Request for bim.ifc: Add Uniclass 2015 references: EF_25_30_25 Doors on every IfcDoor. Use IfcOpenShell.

First a look at what the model holds.

```python
import ifcopenshell

model = ifcopenshell.open("bim.ifc")
print(model.schema)
print("classifications:", [c.Name for c in model.by_type("IfcClassification")])
for ifc_class in ("IfcDoor", "IfcRoof", "IfcStair", "IfcWall", "IfcWindow"):
    print(ifc_class, len(model.by_type(ifc_class)))
```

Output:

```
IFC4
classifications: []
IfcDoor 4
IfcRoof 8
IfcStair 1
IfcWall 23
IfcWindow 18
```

```python
import ifcopenshell
import ifcopenshell.api.classification

model = ifcopenshell.open("bim.ifc")

system = ifcopenshell.api.classification.add_classification(model, classification="Uniclass 2015")

codes = {
    "IfcDoor": ("EF_25_30_25", "Doors"),
}
for ifc_class, (code, name) in codes.items():
    products = model.by_type(ifc_class)
    ifcopenshell.api.classification.add_reference(
        model, products=products, classification=system, identification=code, name=name
    )
    print(code, len(products))

model.write("bim_edited.ifc")
```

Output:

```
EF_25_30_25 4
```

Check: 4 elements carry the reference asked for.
